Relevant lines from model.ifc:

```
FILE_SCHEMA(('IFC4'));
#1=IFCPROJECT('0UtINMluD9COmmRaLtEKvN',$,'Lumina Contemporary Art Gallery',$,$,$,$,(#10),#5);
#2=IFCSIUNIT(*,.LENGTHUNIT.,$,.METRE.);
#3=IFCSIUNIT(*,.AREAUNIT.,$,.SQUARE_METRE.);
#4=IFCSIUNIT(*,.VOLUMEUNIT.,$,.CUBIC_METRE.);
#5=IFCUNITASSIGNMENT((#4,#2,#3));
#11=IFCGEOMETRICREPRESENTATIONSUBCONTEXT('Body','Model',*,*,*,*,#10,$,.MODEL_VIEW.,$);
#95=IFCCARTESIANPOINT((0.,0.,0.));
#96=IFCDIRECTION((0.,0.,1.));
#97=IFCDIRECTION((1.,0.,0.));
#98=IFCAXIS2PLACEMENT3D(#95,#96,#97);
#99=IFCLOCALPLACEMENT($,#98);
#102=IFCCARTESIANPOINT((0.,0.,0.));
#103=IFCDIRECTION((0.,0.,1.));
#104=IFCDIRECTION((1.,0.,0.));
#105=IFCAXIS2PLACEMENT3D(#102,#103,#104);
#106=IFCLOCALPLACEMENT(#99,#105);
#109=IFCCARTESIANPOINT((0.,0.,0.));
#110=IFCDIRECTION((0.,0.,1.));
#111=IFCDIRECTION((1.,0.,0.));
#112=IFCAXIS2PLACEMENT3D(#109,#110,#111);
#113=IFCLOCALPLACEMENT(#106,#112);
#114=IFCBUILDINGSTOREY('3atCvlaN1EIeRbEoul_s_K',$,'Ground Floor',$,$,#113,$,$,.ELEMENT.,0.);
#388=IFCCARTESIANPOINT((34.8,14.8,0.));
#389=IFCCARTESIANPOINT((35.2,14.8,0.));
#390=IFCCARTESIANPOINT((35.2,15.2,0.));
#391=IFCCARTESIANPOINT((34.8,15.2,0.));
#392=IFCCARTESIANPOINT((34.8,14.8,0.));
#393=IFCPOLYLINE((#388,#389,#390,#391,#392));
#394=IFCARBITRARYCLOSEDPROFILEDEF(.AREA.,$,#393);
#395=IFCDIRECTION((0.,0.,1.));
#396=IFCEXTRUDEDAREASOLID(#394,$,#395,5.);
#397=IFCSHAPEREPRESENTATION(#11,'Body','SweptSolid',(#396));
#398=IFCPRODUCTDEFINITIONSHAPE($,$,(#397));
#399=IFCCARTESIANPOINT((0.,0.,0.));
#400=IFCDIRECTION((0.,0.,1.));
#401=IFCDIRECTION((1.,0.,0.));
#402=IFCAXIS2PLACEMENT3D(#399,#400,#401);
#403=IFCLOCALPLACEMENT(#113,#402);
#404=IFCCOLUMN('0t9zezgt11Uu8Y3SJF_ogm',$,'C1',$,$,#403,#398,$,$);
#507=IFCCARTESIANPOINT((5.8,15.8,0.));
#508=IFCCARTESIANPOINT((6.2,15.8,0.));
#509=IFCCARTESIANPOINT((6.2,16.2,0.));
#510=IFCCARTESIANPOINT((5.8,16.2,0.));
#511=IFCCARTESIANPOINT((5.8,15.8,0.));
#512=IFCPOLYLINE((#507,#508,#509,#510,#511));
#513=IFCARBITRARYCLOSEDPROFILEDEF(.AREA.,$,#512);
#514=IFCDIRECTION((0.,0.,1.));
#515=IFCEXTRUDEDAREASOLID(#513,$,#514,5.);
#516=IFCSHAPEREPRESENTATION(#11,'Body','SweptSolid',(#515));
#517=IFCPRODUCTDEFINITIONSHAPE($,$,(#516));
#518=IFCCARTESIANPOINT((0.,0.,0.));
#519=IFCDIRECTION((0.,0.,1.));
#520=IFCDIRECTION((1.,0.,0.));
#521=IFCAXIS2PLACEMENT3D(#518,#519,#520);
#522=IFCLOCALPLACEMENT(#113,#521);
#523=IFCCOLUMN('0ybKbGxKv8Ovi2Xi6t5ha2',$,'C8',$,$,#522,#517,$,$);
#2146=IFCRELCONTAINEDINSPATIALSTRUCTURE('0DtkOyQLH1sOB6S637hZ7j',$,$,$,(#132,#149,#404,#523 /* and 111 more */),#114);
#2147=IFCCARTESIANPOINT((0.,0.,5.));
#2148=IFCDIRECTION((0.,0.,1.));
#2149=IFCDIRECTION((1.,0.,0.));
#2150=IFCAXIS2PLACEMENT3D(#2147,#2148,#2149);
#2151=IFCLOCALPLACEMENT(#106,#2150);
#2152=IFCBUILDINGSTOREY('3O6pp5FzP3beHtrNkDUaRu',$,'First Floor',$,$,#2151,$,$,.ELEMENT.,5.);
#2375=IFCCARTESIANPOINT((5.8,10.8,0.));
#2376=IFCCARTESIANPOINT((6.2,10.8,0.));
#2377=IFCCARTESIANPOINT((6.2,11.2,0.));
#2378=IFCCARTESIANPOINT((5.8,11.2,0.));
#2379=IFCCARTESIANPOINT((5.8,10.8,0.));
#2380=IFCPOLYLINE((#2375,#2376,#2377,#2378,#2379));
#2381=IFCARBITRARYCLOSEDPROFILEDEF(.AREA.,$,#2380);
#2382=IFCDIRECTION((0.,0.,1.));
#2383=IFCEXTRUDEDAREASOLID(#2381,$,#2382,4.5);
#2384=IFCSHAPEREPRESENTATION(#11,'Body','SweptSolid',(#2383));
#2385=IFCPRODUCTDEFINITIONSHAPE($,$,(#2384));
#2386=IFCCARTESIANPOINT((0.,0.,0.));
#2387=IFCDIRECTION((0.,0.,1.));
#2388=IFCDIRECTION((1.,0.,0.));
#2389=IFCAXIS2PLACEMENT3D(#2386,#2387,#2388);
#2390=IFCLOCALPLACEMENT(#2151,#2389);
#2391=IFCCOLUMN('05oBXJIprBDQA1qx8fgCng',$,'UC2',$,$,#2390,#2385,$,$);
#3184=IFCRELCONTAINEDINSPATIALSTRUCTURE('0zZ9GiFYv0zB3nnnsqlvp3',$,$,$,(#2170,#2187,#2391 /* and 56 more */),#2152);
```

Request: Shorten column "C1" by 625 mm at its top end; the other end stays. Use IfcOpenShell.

```python
import ifcopenshell
import ifcopenshell.util.representation
import ifcopenshell.util.unit

model = ifcopenshell.open("model.ifc")
unit_scale = ifcopenshell.util.unit.calculate_unit_scale(model)

member = model.by_guid("0t9zezgt11Uu8Y3SJF_ogm")
change = -0.625 / unit_scale

# The extrusion runs towards the end named, so only its depth changes.
body = ifcopenshell.util.representation.get_representation(member, "Model", "Body")
solid = body.Items[0]
old_length = solid.Depth
solid.Depth += change

print(f"length {old_length:g} -> {solid.Depth:g}")

model.write("model_edited.ifc")
```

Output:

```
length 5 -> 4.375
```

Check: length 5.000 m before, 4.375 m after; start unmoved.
